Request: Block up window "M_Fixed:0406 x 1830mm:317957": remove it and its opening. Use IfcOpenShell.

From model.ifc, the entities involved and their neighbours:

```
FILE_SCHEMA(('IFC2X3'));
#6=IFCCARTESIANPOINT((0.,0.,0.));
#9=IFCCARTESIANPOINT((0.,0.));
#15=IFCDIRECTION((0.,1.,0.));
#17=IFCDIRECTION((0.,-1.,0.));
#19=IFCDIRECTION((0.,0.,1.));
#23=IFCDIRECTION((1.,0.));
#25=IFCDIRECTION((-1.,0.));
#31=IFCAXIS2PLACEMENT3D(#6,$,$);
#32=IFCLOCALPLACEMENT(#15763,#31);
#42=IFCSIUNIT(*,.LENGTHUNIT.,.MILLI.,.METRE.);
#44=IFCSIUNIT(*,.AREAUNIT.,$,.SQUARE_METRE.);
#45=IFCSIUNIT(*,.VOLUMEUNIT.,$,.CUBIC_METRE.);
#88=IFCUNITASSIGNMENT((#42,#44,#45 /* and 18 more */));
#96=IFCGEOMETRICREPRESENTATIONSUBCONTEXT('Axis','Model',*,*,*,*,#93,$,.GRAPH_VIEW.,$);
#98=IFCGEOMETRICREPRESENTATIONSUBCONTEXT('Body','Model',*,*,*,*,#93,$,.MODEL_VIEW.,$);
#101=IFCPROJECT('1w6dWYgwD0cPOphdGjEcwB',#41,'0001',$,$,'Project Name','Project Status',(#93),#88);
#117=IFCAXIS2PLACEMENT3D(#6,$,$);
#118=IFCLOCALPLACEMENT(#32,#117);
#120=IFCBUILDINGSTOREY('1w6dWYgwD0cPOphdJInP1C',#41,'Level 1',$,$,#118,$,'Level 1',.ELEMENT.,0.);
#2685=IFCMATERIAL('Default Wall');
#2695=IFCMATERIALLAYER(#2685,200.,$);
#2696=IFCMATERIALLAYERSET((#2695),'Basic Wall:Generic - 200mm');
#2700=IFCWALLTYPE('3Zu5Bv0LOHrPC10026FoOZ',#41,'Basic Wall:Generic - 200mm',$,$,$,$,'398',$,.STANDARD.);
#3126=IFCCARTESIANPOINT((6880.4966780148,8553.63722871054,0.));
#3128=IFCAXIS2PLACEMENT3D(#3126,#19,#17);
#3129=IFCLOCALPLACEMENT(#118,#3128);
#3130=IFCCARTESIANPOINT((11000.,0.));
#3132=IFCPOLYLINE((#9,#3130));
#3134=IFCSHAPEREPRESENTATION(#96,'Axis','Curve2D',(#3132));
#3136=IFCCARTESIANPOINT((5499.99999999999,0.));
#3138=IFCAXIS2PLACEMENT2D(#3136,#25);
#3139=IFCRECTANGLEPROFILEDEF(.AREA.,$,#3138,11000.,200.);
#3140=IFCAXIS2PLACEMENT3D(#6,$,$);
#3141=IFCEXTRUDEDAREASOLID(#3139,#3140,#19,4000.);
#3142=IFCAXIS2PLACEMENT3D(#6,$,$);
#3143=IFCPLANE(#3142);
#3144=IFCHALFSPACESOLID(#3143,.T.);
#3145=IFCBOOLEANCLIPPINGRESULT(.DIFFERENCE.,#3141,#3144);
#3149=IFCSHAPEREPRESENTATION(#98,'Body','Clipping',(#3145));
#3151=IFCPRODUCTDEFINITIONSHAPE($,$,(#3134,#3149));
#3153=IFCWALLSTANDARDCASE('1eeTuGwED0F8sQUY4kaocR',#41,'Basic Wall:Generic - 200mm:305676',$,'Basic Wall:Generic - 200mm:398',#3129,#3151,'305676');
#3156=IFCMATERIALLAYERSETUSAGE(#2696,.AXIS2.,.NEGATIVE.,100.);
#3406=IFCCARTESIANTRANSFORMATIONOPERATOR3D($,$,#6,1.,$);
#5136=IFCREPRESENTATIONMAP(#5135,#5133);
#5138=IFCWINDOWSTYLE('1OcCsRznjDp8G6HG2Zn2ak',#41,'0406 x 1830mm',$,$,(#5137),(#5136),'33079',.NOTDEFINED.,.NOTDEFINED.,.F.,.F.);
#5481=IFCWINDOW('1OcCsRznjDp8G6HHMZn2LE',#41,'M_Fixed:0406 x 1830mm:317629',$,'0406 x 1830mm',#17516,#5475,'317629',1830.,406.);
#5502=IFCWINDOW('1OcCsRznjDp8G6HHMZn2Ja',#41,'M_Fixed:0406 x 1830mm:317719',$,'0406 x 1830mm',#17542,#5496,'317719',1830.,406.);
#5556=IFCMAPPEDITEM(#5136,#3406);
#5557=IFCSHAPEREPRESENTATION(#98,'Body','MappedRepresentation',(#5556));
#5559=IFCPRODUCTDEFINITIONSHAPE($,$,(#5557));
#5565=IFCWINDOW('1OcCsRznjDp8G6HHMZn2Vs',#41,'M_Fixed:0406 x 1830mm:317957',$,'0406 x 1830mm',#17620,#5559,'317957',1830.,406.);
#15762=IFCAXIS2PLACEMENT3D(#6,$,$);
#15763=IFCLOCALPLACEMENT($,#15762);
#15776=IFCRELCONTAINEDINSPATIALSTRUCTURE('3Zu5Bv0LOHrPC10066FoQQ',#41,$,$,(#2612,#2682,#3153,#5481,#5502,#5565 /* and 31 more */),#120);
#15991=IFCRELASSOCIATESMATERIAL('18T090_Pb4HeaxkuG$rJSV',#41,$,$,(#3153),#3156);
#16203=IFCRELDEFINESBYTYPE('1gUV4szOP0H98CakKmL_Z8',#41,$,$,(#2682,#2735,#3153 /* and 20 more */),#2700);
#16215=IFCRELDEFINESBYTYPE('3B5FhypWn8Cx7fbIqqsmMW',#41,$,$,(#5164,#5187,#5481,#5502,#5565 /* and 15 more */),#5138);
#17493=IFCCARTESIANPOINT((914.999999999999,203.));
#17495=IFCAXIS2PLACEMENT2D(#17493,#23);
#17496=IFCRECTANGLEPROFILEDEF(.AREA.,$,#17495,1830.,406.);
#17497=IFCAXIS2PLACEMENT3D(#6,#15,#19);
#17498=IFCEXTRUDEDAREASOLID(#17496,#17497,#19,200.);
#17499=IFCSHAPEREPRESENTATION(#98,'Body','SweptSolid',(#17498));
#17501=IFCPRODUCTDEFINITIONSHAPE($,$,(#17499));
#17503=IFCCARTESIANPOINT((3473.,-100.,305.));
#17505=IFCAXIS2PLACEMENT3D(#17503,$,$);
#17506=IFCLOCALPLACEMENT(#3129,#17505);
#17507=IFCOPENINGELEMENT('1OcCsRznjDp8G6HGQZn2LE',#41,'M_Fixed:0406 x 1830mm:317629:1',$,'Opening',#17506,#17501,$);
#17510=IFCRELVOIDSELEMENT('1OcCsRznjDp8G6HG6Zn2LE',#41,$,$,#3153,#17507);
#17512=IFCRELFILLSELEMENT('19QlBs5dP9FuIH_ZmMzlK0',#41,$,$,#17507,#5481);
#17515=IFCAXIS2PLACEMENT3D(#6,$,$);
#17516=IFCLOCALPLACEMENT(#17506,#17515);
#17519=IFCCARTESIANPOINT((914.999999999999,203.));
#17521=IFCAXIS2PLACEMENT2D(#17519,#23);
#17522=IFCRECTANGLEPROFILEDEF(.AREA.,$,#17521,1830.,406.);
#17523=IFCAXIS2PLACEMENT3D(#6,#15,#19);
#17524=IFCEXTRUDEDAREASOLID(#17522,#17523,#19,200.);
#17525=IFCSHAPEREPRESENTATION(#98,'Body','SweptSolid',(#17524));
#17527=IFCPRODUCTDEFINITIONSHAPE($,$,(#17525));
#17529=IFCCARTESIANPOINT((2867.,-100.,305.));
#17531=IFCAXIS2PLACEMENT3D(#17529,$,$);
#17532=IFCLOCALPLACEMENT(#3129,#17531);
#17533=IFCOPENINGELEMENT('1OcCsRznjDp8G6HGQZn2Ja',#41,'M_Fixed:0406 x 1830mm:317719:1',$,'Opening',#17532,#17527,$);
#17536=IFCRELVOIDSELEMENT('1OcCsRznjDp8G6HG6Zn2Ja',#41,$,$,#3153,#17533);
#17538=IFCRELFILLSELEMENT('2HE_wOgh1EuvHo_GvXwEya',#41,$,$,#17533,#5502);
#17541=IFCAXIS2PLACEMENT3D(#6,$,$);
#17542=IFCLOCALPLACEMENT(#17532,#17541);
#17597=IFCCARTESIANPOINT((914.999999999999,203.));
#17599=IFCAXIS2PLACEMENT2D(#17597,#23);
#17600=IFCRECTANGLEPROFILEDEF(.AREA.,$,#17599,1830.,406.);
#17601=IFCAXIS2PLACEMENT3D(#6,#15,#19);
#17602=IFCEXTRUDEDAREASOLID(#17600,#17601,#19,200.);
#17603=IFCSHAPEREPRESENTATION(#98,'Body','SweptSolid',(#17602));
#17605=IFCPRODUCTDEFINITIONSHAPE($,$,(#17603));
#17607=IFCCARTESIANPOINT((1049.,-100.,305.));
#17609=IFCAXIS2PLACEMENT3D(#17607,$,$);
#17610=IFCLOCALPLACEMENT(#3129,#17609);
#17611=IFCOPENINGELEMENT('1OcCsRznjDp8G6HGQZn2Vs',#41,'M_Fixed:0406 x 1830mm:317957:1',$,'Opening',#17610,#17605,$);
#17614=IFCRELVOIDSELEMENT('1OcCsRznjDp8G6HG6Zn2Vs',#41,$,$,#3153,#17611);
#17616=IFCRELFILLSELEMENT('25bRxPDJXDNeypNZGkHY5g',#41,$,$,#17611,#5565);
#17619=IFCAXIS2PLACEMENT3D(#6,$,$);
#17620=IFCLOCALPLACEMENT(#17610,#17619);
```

```python
import ifcopenshell
import ifcopenshell.api.feature
import ifcopenshell.api.root
import ifcopenshell.geom
import ifcopenshell.util.shape

model = ifcopenshell.open("model.ifc")
settings = ifcopenshell.geom.settings()


def volume(element):
    """Net volume in cubic metres, openings subtracted."""
    shape = ifcopenshell.geom.create_shape(settings, element)
    return ifcopenshell.util.shape.get_volume(shape.geometry)


window = model.by_id(5565)
opening = window.FillsVoids[0].RelatingOpeningElement
wall = opening.VoidsElements[0].RelatingBuildingElement
before = volume(wall)

ifcopenshell.api.root.remove_product(model, product=window)
ifcopenshell.api.feature.remove_feature(model, feature=opening)

after = volume(wall)

print(f"wall volume {before:.3f} -> {after:.3f} m3")

model.write("model_updated.ifc")
```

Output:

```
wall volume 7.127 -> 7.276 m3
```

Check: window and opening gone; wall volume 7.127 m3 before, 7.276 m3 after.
